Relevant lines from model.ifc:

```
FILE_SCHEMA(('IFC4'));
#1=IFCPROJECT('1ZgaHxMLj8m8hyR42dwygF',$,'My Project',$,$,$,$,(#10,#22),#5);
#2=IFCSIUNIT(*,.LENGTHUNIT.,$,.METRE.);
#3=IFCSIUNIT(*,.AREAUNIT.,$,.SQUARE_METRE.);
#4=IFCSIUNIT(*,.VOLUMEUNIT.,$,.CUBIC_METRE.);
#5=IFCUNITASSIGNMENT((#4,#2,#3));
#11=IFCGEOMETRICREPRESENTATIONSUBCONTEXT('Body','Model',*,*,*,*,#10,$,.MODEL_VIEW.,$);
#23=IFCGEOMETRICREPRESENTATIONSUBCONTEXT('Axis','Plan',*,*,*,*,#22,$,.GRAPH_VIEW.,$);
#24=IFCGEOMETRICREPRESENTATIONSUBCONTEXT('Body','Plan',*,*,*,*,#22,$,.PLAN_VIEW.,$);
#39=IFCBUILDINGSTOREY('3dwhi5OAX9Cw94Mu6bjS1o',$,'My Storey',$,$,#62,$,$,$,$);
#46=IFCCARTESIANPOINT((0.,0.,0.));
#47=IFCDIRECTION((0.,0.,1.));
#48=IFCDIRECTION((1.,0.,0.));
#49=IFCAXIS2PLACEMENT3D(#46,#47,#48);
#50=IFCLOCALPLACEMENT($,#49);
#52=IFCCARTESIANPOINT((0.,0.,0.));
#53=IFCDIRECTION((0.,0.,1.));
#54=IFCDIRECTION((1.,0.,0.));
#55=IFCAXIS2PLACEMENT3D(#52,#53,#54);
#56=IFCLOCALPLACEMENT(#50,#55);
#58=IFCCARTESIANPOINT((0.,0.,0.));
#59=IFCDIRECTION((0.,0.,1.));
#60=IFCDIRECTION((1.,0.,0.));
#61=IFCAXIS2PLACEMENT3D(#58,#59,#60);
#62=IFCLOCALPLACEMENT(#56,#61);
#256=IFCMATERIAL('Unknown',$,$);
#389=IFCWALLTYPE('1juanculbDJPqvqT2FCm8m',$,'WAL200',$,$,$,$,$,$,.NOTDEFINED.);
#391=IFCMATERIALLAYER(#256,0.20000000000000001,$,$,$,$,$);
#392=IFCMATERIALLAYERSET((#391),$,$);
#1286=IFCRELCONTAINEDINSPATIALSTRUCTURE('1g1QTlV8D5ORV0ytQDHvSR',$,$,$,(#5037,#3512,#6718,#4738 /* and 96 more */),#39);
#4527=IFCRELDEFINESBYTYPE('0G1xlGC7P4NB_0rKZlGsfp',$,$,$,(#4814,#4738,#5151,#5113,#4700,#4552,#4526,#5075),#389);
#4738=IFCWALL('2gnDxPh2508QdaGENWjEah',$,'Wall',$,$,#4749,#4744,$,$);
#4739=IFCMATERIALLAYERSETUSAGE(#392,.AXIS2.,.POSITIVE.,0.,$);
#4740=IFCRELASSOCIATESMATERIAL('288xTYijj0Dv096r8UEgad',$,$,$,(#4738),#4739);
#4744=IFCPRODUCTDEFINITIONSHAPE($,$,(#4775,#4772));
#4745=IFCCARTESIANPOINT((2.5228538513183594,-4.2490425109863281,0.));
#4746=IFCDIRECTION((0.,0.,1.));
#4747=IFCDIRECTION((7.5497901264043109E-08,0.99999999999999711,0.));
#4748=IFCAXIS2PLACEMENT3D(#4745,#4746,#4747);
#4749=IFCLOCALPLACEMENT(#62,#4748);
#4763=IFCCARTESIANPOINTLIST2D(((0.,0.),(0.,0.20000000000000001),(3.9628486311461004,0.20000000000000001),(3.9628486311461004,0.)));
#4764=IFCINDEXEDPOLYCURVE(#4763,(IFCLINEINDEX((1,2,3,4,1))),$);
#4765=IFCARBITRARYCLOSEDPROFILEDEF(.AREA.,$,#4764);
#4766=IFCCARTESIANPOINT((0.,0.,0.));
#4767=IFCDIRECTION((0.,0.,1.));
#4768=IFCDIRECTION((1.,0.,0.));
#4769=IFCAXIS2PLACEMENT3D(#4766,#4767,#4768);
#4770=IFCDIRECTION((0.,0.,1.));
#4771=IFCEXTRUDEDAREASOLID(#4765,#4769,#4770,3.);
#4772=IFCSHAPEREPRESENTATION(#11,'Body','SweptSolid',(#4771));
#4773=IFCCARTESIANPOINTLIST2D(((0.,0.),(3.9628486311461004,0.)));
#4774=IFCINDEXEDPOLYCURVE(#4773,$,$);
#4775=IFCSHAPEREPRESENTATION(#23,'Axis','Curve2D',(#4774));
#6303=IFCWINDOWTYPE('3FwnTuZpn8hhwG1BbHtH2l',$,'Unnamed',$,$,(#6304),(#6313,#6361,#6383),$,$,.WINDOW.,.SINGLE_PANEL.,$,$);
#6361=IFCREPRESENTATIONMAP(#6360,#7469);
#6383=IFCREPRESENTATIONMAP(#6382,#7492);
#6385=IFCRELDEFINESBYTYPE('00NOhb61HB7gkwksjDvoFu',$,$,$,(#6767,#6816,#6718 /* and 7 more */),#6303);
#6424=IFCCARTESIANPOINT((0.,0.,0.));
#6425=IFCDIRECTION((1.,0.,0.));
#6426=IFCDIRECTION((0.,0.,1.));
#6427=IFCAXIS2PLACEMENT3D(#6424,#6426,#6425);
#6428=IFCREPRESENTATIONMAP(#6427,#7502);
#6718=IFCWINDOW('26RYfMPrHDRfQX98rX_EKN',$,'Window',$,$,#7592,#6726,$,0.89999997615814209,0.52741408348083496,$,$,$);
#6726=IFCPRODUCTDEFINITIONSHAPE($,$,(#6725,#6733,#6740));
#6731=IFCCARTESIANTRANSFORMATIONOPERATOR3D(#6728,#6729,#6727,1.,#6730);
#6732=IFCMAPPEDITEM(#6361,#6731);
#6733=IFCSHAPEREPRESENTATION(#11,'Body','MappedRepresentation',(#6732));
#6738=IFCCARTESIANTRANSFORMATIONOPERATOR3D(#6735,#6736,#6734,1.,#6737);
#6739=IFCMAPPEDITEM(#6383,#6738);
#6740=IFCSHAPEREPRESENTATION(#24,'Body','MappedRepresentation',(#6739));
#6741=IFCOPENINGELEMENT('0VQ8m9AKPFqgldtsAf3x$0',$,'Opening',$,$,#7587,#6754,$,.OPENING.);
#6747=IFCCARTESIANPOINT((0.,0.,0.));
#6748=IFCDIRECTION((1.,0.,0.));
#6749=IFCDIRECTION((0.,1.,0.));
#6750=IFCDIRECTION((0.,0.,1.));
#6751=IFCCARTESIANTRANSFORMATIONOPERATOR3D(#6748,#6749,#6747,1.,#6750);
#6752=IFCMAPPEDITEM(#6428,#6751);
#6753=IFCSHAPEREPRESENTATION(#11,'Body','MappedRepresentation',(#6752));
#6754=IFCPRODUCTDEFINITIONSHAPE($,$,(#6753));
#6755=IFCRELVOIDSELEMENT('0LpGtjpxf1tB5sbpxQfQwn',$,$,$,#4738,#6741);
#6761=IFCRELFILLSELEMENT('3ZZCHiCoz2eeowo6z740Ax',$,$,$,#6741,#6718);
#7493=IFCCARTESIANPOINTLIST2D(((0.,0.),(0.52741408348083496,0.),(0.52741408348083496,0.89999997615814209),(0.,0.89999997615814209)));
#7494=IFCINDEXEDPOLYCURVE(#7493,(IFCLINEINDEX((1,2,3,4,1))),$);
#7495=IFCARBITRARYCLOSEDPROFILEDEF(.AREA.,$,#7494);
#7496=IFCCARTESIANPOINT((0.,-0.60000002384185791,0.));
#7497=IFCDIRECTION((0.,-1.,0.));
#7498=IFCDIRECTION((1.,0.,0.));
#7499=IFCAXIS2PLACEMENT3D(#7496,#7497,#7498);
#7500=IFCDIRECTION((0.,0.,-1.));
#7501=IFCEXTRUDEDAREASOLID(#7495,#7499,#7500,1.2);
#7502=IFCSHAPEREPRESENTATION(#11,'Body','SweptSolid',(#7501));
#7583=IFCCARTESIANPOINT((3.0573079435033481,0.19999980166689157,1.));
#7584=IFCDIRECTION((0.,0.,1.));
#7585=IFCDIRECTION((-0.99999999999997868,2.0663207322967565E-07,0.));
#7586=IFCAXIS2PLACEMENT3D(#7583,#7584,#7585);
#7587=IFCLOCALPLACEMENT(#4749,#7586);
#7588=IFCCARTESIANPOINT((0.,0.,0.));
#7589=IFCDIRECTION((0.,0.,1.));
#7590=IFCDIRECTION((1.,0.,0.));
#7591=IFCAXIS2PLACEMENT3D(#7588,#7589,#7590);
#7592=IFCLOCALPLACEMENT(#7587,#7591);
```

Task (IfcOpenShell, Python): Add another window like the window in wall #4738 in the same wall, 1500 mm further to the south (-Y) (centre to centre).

```python
import ifcopenshell
import ifcopenshell.api.feature
import ifcopenshell.api.geometry
import ifcopenshell.api.root
import ifcopenshell.geom
import ifcopenshell.util.element
import ifcopenshell.util.placement
import ifcopenshell.util.shape
import ifcopenshell.util.unit

model = ifcopenshell.open("model.ifc")
unit_scale = ifcopenshell.util.unit.calculate_unit_scale(model)
settings = ifcopenshell.geom.settings()


def volume(element):
    """Net volume in cubic metres, openings subtracted."""
    shape = ifcopenshell.geom.create_shape(settings, element)
    return ifcopenshell.util.shape.get_volume(shape.geometry)


window = model.by_guid("26RYfMPrHDRfQX98rX_EKN")
opening = window.FillsVoids[0].RelatingOpeningElement
wall = opening.VoidsElements[0].RelatingBuildingElement
before = volume(wall)
shift = ifcopenshell.util.placement.get_local_placement(wall.ObjectPlacement)[:3, 0] * -1.5 / unit_scale

# copy_class copies the void relationship, type, container and properties, but no geometry.
new_opening = ifcopenshell.api.root.copy_class(model, product=opening)
new_opening.Representation = ifcopenshell.util.element.copy_deep(
    model, opening.Representation, exclude=["IfcGeometricRepresentationContext", "IfcRepresentationMap"]
)
new_window = ifcopenshell.api.root.copy_class(model, product=window)
new_window.Representation = ifcopenshell.util.element.copy_deep(
    model, window.Representation, exclude=["IfcGeometricRepresentationContext", "IfcRepresentationMap"]
)
ifcopenshell.api.feature.add_filling(model, opening=new_opening, element=new_window)

for old, new in ((opening, new_opening), (window, new_window)):
    matrix = ifcopenshell.util.placement.get_local_placement(old.ObjectPlacement)
    matrix[:3, 3] += shift
    ifcopenshell.api.geometry.edit_object_placement(model, product=new, matrix=matrix, is_si=False)

after = volume(wall)

print(f"wall volume {before:.3f} -> {after:.3f} m3")

model.write("model_v2.ifc")
```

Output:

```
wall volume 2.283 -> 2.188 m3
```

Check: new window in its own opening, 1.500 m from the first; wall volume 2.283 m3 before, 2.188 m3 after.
